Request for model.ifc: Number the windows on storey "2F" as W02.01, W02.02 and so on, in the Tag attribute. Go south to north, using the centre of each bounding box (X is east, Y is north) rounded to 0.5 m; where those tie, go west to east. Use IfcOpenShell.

First a look at what the model holds.

```python
import ifcopenshell
import ifcopenshell.util.element
import ifcopenshell.util.placement

model = ifcopenshell.open("model.ifc")
print(model.schema)
storey = next(s for s in model.by_type("IfcBuildingStorey") if s.Name == "2F")
windows = [e for e in ifcopenshell.util.element.get_decomposition(storey) if e.is_a("IfcWindow")]
for e in sorted(windows, key=lambda e: e.id()):
    origin = ifcopenshell.util.placement.get_local_placement(e.ObjectPlacement)[:3, 3]
    print(e.id(), e.Tag, e.Name, origin.round(2) + 0.0, sep=" | ")
```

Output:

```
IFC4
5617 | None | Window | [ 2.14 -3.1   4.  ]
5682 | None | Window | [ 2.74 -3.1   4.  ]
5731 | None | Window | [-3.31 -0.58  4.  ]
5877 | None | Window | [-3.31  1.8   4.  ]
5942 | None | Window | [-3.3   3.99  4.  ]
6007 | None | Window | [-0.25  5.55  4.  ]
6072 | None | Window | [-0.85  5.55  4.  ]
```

```python
import ifcopenshell
import ifcopenshell.geom
import ifcopenshell.util.element
import ifcopenshell.util.shape

model = ifcopenshell.open("model.ifc")
settings = ifcopenshell.geom.settings()
settings.set("use-world-coords", True)


def centre(element):
    shape = ifcopenshell.geom.create_shape(settings, element)
    return ifcopenshell.util.shape.get_bbox_centroid(shape.geometry)


storey = next(s for s in model.by_type("IfcBuildingStorey") if s.Name == "2F")
windows = [e for e in ifcopenshell.util.element.get_decomposition(storey) if e.is_a("IfcWindow")]

# Insertion points can sit at a corner or the storey origin, so sort by the geometry (in metres).
centres = {e: centre(e) for e in windows}
windows.sort(key=lambda e: (round(centres[e][1] / 0.5), centres[e][0]))

for i, e in enumerate(windows, start=1):
    number = f"W02.{i:02d}"
    e.Tag = number
    print(e.id(), number)

model.write("model_v2.ifc")
```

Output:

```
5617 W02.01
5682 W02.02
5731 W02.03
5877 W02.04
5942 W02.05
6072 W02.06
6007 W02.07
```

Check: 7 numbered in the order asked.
